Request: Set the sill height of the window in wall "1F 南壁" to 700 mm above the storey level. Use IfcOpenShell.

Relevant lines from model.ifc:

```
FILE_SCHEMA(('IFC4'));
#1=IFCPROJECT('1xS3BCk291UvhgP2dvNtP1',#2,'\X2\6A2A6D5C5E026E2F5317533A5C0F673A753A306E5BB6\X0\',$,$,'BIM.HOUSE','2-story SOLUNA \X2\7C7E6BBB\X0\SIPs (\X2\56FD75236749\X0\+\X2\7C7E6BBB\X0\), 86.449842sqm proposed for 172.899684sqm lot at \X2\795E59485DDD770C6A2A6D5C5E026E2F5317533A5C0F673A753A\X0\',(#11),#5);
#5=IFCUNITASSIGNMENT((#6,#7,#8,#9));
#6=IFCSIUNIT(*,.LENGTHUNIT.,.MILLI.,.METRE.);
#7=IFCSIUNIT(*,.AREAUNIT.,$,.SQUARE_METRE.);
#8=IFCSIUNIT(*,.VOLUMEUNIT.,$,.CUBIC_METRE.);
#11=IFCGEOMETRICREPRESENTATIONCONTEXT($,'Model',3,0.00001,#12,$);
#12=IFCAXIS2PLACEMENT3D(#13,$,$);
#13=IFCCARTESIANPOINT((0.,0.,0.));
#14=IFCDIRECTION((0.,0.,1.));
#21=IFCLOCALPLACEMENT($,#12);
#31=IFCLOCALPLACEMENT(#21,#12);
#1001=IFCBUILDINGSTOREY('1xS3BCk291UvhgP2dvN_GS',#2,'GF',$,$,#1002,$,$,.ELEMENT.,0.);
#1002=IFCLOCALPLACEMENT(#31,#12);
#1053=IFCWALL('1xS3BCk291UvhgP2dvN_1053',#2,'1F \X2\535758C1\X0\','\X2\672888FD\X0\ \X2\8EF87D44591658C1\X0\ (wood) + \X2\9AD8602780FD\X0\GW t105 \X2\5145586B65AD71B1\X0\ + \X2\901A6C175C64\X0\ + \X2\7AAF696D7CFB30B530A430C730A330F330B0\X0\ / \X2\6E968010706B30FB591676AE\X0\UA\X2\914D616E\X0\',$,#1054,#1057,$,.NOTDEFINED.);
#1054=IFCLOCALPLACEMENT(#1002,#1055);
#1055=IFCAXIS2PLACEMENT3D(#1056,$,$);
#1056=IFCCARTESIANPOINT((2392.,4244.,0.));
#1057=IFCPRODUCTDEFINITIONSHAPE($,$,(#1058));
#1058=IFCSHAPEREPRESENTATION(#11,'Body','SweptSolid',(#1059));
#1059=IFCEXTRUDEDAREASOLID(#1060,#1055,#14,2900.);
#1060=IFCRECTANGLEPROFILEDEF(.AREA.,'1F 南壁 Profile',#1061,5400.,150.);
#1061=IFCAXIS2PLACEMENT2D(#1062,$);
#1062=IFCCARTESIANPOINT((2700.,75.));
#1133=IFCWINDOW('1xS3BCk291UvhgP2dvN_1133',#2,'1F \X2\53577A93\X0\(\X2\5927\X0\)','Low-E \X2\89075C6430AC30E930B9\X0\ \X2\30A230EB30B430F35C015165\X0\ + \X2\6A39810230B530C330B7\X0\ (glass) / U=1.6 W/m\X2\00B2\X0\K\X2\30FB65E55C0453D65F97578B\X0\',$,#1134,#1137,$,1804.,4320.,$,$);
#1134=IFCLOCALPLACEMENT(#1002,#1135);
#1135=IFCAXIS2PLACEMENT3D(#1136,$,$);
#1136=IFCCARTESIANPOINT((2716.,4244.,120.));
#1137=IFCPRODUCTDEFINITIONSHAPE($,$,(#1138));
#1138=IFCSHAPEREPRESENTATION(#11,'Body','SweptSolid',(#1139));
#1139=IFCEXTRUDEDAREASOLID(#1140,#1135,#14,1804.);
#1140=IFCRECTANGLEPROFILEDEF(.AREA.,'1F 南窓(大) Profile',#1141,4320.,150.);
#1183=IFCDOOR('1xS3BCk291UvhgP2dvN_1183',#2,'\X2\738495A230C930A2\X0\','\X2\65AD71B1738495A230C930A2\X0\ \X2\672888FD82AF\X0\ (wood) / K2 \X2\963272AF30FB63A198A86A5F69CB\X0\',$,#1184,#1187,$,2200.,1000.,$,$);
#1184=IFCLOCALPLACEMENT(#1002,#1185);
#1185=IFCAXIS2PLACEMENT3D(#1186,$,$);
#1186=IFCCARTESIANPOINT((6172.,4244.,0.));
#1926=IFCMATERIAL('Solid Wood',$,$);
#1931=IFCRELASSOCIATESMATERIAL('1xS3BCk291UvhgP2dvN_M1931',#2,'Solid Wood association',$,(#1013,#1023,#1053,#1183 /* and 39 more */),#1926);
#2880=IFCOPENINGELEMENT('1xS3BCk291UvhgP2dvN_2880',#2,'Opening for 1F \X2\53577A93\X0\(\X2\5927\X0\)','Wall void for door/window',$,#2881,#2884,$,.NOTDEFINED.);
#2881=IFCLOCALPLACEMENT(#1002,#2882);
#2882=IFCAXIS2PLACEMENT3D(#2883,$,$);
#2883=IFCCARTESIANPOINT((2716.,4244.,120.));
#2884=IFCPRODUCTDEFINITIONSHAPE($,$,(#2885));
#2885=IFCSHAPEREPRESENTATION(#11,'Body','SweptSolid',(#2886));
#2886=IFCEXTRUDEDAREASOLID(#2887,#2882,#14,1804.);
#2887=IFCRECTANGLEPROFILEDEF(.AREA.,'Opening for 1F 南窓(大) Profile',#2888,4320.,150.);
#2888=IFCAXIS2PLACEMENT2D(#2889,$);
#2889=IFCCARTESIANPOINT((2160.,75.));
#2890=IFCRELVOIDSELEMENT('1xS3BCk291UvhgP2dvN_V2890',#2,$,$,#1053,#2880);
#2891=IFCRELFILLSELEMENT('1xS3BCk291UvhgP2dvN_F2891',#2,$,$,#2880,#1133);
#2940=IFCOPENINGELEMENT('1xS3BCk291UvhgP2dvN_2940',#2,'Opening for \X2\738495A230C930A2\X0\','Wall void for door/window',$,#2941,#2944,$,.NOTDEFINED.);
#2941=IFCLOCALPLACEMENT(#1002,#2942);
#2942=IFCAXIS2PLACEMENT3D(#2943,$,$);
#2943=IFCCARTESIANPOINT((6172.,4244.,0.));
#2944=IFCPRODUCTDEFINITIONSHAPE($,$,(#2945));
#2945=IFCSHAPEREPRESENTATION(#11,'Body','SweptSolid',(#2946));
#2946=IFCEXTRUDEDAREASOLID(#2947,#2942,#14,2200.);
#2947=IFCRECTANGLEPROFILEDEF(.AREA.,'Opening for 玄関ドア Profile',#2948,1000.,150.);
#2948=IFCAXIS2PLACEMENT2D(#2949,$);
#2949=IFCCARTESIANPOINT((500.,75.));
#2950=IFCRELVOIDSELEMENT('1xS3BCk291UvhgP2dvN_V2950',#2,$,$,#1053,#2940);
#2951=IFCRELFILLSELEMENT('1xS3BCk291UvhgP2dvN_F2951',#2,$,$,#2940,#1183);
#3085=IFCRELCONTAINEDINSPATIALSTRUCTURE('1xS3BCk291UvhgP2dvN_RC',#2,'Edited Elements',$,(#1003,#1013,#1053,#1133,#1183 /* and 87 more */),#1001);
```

```python
import numpy as np
import ifcopenshell
import ifcopenshell.api.geometry
import ifcopenshell.geom
import ifcopenshell.util.element
import ifcopenshell.util.placement
import ifcopenshell.util.shape
import ifcopenshell.util.unit

model = ifcopenshell.open("model.ifc")
unit_scale = ifcopenshell.util.unit.calculate_unit_scale(model)

window = model.by_guid("1xS3BCk291UvhgP2dvN_1133")
opening = window.FillsVoids[0].RelatingOpeningElement
storey = ifcopenshell.util.element.get_container(window, ifc_class="IfcBuildingStorey")
level = ifcopenshell.util.placement.get_local_placement(storey.ObjectPlacement)[2, 3]

# The opening's origin need not be at the sill, so measure its lowest point.
shape = ifcopenshell.geom.create_shape(ifcopenshell.geom.settings(), opening)
bottom = ifcopenshell.util.shape.get_shape_bottom_elevation(shape, shape.geometry) / unit_scale
dz = level + 700.0 - bottom

shift = np.array([0.0, 0.0, dz])
# The window is not placed relative to its opening, so move both.
for product in (opening, window):
    matrix = ifcopenshell.util.placement.get_local_placement(product.ObjectPlacement)
    matrix[:3, 3] += shift
    ifcopenshell.api.geometry.edit_object_placement(model, product=product, matrix=matrix, is_si=False)

print(f"moved by {dz * unit_scale:+.3f} m")

model.write("model-out.ifc")
```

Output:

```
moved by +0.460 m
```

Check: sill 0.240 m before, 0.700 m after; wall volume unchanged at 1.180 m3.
